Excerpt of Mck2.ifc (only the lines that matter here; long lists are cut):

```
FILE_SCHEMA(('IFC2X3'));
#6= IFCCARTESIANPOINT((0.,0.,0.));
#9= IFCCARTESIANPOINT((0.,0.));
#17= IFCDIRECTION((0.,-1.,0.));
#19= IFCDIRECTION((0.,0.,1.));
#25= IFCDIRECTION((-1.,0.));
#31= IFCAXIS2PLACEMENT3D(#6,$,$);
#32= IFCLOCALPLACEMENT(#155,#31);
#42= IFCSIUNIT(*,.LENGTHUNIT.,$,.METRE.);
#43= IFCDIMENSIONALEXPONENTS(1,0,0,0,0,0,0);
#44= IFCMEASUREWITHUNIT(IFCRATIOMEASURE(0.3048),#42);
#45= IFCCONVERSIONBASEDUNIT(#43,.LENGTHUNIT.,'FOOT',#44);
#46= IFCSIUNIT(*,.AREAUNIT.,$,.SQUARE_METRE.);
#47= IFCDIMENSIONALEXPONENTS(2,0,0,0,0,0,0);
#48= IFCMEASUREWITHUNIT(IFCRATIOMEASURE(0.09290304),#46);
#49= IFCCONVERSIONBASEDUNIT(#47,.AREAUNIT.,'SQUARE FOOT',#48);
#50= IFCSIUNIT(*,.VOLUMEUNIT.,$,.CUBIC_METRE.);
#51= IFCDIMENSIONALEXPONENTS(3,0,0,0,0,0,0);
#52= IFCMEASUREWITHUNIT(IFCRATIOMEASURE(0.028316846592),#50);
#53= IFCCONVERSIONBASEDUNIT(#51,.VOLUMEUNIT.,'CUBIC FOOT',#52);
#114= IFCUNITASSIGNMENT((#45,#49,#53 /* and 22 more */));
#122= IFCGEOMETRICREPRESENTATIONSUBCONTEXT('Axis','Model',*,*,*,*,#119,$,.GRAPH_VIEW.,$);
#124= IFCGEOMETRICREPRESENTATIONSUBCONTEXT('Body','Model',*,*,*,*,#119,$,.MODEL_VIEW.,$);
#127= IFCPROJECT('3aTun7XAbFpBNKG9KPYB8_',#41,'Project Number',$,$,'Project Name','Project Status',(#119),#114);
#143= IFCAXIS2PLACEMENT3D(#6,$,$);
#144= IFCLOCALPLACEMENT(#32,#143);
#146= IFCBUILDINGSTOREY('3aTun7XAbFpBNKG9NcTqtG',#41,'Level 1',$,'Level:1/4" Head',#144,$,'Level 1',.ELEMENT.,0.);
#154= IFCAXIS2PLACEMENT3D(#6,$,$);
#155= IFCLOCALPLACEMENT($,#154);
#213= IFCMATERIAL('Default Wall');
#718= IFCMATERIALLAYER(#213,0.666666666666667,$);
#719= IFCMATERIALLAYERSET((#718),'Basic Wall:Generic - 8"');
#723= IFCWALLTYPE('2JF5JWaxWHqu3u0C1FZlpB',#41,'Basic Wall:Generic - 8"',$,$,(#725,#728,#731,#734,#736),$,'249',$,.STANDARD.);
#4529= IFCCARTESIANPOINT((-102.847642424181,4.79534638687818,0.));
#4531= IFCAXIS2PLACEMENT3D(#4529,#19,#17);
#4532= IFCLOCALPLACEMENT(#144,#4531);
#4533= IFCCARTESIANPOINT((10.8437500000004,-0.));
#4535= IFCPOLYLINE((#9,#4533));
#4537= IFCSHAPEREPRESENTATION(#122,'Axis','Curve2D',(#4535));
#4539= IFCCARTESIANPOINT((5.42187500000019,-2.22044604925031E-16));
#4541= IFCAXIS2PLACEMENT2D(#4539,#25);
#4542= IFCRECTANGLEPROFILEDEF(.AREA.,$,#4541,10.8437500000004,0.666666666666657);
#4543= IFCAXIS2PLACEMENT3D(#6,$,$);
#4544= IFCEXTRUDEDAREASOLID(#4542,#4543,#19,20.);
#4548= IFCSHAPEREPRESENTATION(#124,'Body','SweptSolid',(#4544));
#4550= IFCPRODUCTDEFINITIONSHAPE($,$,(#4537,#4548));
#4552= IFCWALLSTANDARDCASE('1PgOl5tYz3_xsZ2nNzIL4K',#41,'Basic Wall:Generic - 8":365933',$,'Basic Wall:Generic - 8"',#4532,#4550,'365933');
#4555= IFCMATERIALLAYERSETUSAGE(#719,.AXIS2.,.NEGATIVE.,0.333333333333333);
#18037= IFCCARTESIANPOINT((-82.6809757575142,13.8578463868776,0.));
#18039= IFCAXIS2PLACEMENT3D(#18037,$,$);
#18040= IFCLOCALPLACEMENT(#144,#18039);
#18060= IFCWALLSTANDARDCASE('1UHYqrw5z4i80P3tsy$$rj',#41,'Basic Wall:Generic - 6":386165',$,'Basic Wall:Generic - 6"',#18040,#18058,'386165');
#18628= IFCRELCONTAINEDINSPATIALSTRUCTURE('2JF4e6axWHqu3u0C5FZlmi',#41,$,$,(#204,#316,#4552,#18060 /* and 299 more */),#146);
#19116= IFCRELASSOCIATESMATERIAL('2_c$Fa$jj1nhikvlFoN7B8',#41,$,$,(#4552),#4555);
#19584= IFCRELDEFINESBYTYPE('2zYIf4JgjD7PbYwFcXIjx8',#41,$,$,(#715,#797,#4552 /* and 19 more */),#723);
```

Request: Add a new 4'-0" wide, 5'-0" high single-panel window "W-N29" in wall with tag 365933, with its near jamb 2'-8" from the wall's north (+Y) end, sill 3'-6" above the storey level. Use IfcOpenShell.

```python
import numpy as np
import ifcopenshell
import ifcopenshell.api.feature
import ifcopenshell.api.geometry
import ifcopenshell.api.root
import ifcopenshell.api.spatial
import ifcopenshell.api.type
import ifcopenshell.geom
import ifcopenshell.util.element
import ifcopenshell.util.placement
import ifcopenshell.util.representation
import ifcopenshell.util.shape
import ifcopenshell.util.unit

model = ifcopenshell.open("Mck2.ifc")
unit_scale = ifcopenshell.util.unit.calculate_unit_scale(model)
settings = ifcopenshell.geom.settings()


def volume(element):
    """Net volume in cubic metres, openings subtracted."""
    shape = ifcopenshell.geom.create_shape(settings, element)
    return ifcopenshell.util.shape.get_volume(shape.geometry)


wall = model.by_id(4552)
storey = ifcopenshell.util.element.get_container(wall, ifc_class="IfcBuildingStorey")
context = ifcopenshell.util.representation.get_context(model, "Model", "Body", "MODEL_VIEW")
before = volume(wall)

width, height, from_end, sill = 1.2192, 1.524, 0.8128, 1.0668  # metres

# The wall runs along its own X axis, and the end named is its -X end.
wall_shape = ifcopenshell.geom.create_shape(settings, wall)
x, y, z = ifcopenshell.util.shape.get_vertices(wall_shape.geometry).T
start = x.min() + from_end
face, thickness = float(y.min()), float(y.max() - y.min())
wall_matrix = ifcopenshell.util.placement.get_local_placement(wall.ObjectPlacement)
level = ifcopenshell.util.placement.get_local_placement(storey.ObjectPlacement)[2, 3]


def in_wall(x, y):
    """Placement at x, y metres in the wall's axes, at sill height."""
    matrix = wall_matrix.copy()
    matrix[:, 3] = wall_matrix @ np.array([x / unit_scale, y / unit_scale, 0.0, 1.0])
    matrix[2, 3] = level + sill / unit_scale
    return matrix


# Opening: a box that overshoots both wall faces by 50 mm.
opening = ifcopenshell.api.root.create_entity(model, ifc_class="IfcOpeningElement")
box = ifcopenshell.api.geometry.add_wall_representation(
    model, context=context, length=width, height=height, thickness=thickness + 0.1
)
ifcopenshell.api.geometry.assign_representation(model, product=opening, representation=box)
ifcopenshell.api.geometry.edit_object_placement(model, product=opening, matrix=in_wall(start, face - 0.05), is_si=False)
ifcopenshell.api.feature.add_feature(model, feature=opening, element=wall)

window = ifcopenshell.api.root.create_entity(model, ifc_class="IfcWindow", name="W-N29")
window.OverallWidth, window.OverallHeight = width / unit_scale, height / unit_scale
body = ifcopenshell.api.geometry.add_window_representation(
    model,
    context=context,
    overall_width=window.OverallWidth,
    overall_height=window.OverallHeight,
    partition_type="SINGLE_PANEL",
)
ifcopenshell.api.geometry.assign_representation(model, product=window, representation=body)
ifcopenshell.api.spatial.assign_container(model, products=[window], relating_structure=storey)
fills = ifcopenshell.api.feature.add_filling(model, opening=opening, element=window)
fills.OwnerHistory = window.OwnerHistory  # required in IFC2X3

# IFC2X3 keeps the operation on the window style.
style = ifcopenshell.api.root.create_entity(model, ifc_class="IfcWindowStyle", name="W-N29")
style.OperationType, style.ConstructionType = "SINGLE_PANEL", "NOTDEFINED"
style.ParameterTakesPrecedence = style.Sizeable = False
ifcopenshell.api.type.assign_type(model, related_objects=[window], relating_type=style)

# Centre the window in the wall's thickness.
ifcopenshell.api.geometry.edit_object_placement(model, product=window, matrix=in_wall(start, face), is_si=False)
window_shape = ifcopenshell.geom.create_shape(settings, window)
depth = ifcopenshell.util.shape.get_vertices(window_shape.geometry)[:, 1]
offset = face + thickness / 2 - (depth.min() + depth.max()) / 2
ifcopenshell.api.geometry.edit_object_placement(model, product=window, matrix=in_wall(start, offset), is_si=False)

after = volume(wall)

print(f"wall volume {before:.3f} -> {after:.3f} m3")

model.write("Mck2_rev.ifc")
```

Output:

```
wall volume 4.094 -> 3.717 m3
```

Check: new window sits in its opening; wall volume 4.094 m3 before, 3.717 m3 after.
